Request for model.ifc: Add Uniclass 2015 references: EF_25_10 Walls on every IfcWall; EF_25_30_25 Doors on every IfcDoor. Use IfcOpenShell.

First a look at what the model holds.

```python
import ifcopenshell

model = ifcopenshell.open("model.ifc")
print(model.schema)
print("classifications:", [c.Name for c in model.by_type("IfcClassification")])
for ifc_class in ("IfcDoor", "IfcRoof", "IfcStair", "IfcWall", "IfcWindow"):
    print(ifc_class, len(model.by_type(ifc_class)))
```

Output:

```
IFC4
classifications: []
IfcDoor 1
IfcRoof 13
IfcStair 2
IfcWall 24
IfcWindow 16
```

```python
import ifcopenshell
import ifcopenshell.api.classification

model = ifcopenshell.open("model.ifc")

system = ifcopenshell.api.classification.add_classification(model, classification="Uniclass 2015")

codes = {
    "IfcWall": ("EF_25_10", "Walls"),
    "IfcDoor": ("EF_25_30_25", "Doors"),
}
for ifc_class, (code, name) in codes.items():
    products = model.by_type(ifc_class)
    ifcopenshell.api.classification.add_reference(
        model, products=products, classification=system, identification=code, name=name
    )
    print(code, len(products))

model.write("model_v2.ifc")
```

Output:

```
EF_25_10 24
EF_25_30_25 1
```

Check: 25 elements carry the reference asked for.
